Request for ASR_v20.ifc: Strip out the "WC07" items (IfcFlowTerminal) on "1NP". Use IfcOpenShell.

First a look at what the model holds.

```python
import ifcopenshell
import ifcopenshell.util.element

model = ifcopenshell.open("ASR_v20.ifc")
print(model.schema)
storey = next(s for s in model.by_type("IfcBuildingStorey") if s.Name == "1NP")
terminals = [e for e in ifcopenshell.util.element.get_decomposition(storey) if e.is_a("IfcFlowTerminal")]
seen = {}
for e in terminals:
    element_type = ifcopenshell.util.element.get_type(e)
    name = element_type.Name if element_type not in (None, e) else None
    seen[name] = seen.get(name, 0) + 1
for name, count in sorted(seen.items(), key=str):
    print(count, "x", name)
```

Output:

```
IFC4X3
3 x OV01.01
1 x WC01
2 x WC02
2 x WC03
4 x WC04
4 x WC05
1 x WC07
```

```python
import ifcopenshell
import ifcopenshell.api.root
import ifcopenshell.util.element

model = ifcopenshell.open("ASR_v20.ifc")

storey = next(s for s in model.by_type("IfcBuildingStorey") if s.Name == "1NP")
terminals = [e for e in ifcopenshell.util.element.get_decomposition(storey) if e.is_a("IfcFlowTerminal")]
targets = [e for e in terminals if (t := ifcopenshell.util.element.get_type(e)) not in (None, e) and t.Name == "WC07"]

for e in targets:
    ifcopenshell.api.root.remove_product(model, product=e)
print(len(targets), "removed")

model.write("ASR_v20_edited.ifc")
```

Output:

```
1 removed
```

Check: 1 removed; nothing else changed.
